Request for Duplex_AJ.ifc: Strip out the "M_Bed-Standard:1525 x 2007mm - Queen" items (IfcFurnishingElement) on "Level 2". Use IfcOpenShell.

First a look at what the model holds.

```python
import ifcopenshell
import ifcopenshell.util.element

model = ifcopenshell.open("Duplex_AJ.ifc")
print(model.schema)
storey = next(s for s in model.by_type("IfcBuildingStorey") if s.Name == "Level 2")
furniture = [e for e in ifcopenshell.util.element.get_decomposition(storey) if e.is_a("IfcFurnishingElement")]
seen = {}
for e in furniture:
    element_type = ifcopenshell.util.element.get_type(e)
    name = element_type.Name if element_type not in (None, e) else None
    seen[name] = seen.get(name, 0) + 1
for name, count in sorted(seen.items(), key=str):
    print(count, "x", name)
```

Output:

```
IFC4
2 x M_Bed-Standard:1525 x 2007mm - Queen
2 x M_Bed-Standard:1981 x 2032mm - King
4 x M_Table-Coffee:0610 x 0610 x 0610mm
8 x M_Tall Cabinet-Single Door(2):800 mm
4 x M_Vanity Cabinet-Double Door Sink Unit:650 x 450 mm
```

```python
import ifcopenshell
import ifcopenshell.api.root
import ifcopenshell.util.element

model = ifcopenshell.open("Duplex_AJ.ifc")

storey = next(s for s in model.by_type("IfcBuildingStorey") if s.Name == "Level 2")
furniture = [e for e in ifcopenshell.util.element.get_decomposition(storey) if e.is_a("IfcFurnishingElement")]
targets = [e for e in furniture if (t := ifcopenshell.util.element.get_type(e)) not in (None, e) and t.Name == "M_Bed-Standard:1525 x 2007mm - Queen"]

for e in targets:
    ifcopenshell.api.root.remove_product(model, product=e)
print(len(targets), "removed")

model.write("Duplex_AJ_edited.ifc")
```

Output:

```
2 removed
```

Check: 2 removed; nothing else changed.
